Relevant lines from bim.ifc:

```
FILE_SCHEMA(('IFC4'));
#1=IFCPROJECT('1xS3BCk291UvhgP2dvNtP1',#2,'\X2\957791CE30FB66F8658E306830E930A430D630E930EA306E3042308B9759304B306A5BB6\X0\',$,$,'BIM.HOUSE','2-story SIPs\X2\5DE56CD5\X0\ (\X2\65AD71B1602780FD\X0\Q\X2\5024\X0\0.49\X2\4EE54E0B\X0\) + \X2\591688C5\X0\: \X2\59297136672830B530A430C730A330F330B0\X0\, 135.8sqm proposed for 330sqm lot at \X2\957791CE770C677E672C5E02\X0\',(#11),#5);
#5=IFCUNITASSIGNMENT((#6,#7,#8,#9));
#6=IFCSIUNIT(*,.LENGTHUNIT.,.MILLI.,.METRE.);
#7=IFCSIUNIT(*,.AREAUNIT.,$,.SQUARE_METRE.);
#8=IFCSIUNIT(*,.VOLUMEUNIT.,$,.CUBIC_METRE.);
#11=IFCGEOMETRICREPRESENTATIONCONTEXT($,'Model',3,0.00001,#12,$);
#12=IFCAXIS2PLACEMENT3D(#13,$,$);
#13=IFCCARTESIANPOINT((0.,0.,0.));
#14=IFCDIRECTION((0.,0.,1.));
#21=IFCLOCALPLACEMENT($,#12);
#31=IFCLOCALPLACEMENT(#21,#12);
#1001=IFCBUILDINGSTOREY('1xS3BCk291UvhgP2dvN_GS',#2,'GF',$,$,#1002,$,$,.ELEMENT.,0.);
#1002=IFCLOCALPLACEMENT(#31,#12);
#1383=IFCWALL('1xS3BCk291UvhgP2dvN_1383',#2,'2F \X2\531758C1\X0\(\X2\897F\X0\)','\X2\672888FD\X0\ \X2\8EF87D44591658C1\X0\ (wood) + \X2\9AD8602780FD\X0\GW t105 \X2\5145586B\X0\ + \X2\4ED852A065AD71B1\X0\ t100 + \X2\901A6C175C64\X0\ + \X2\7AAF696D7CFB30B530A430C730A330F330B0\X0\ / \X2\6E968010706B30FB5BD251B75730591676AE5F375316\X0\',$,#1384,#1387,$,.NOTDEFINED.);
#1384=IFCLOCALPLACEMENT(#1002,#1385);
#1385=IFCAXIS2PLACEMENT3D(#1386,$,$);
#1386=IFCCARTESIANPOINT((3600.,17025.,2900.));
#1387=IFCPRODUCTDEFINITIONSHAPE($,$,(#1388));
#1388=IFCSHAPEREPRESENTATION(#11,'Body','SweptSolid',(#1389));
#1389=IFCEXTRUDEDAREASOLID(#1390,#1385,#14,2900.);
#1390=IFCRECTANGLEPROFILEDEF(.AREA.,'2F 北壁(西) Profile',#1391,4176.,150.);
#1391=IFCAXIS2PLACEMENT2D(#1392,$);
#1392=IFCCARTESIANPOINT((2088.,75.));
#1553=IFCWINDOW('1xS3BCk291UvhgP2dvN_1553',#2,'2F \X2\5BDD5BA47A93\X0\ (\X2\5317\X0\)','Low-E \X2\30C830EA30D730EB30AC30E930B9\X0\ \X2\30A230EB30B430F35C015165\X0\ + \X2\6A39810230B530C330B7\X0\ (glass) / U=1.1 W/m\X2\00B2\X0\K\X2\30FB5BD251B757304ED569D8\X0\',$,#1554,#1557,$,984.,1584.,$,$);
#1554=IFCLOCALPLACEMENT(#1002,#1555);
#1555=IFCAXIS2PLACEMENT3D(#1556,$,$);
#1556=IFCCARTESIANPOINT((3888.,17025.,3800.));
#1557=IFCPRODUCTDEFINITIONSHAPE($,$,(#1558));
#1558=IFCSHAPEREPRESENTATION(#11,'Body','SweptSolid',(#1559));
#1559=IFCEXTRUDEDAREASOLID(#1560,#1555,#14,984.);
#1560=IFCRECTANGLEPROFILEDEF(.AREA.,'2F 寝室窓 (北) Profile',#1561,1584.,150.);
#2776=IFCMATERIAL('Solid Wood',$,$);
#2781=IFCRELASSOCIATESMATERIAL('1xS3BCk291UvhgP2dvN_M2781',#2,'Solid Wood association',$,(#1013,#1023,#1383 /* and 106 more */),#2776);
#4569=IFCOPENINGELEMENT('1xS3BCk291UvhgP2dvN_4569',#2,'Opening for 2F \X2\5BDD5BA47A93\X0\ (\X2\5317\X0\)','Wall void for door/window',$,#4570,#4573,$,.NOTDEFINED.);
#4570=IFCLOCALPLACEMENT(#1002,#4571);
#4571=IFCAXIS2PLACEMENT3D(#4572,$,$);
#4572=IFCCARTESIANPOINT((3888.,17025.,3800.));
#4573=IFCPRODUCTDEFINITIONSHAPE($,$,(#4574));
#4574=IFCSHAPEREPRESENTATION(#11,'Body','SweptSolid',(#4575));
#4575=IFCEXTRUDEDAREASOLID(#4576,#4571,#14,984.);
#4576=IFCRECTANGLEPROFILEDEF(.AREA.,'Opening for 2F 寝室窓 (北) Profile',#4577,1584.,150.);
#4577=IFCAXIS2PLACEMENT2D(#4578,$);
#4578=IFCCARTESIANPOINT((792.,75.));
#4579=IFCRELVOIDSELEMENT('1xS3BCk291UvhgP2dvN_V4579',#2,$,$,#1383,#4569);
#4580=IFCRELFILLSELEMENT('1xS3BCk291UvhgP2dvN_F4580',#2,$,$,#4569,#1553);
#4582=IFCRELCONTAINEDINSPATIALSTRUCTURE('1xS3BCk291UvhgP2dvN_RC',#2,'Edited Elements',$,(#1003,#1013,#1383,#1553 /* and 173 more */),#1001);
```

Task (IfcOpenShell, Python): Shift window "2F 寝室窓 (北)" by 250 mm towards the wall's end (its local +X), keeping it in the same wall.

```python
import ifcopenshell
import ifcopenshell.api.geometry
import ifcopenshell.util.placement
import ifcopenshell.util.unit

model = ifcopenshell.open("bim.ifc")
unit_scale = ifcopenshell.util.unit.calculate_unit_scale(model)

window = model.by_id(1553)
opening = window.FillsVoids[0].RelatingOpeningElement
wall = opening.VoidsElements[0].RelatingBuildingElement

wall_matrix = ifcopenshell.util.placement.get_local_placement(wall.ObjectPlacement)
shift = wall_matrix[:3, 0] * 0.25 / unit_scale
before = ifcopenshell.util.placement.get_local_placement(window.ObjectPlacement)[:3, 3].copy()

# The window is not placed relative to its opening, so move both.
for product in (opening, window):
    matrix = ifcopenshell.util.placement.get_local_placement(product.ObjectPlacement)
    matrix[:3, 3] += shift
    ifcopenshell.api.geometry.edit_object_placement(model, product=product, matrix=matrix, is_si=False)

after = ifcopenshell.util.placement.get_local_placement(window.ObjectPlacement)[:3, 3]
print("window moved by", (after - before).round(3) + 0.0)

model.write("bim_rev.ifc")
```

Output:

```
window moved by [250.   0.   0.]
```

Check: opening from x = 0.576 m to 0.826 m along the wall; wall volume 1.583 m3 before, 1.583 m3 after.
